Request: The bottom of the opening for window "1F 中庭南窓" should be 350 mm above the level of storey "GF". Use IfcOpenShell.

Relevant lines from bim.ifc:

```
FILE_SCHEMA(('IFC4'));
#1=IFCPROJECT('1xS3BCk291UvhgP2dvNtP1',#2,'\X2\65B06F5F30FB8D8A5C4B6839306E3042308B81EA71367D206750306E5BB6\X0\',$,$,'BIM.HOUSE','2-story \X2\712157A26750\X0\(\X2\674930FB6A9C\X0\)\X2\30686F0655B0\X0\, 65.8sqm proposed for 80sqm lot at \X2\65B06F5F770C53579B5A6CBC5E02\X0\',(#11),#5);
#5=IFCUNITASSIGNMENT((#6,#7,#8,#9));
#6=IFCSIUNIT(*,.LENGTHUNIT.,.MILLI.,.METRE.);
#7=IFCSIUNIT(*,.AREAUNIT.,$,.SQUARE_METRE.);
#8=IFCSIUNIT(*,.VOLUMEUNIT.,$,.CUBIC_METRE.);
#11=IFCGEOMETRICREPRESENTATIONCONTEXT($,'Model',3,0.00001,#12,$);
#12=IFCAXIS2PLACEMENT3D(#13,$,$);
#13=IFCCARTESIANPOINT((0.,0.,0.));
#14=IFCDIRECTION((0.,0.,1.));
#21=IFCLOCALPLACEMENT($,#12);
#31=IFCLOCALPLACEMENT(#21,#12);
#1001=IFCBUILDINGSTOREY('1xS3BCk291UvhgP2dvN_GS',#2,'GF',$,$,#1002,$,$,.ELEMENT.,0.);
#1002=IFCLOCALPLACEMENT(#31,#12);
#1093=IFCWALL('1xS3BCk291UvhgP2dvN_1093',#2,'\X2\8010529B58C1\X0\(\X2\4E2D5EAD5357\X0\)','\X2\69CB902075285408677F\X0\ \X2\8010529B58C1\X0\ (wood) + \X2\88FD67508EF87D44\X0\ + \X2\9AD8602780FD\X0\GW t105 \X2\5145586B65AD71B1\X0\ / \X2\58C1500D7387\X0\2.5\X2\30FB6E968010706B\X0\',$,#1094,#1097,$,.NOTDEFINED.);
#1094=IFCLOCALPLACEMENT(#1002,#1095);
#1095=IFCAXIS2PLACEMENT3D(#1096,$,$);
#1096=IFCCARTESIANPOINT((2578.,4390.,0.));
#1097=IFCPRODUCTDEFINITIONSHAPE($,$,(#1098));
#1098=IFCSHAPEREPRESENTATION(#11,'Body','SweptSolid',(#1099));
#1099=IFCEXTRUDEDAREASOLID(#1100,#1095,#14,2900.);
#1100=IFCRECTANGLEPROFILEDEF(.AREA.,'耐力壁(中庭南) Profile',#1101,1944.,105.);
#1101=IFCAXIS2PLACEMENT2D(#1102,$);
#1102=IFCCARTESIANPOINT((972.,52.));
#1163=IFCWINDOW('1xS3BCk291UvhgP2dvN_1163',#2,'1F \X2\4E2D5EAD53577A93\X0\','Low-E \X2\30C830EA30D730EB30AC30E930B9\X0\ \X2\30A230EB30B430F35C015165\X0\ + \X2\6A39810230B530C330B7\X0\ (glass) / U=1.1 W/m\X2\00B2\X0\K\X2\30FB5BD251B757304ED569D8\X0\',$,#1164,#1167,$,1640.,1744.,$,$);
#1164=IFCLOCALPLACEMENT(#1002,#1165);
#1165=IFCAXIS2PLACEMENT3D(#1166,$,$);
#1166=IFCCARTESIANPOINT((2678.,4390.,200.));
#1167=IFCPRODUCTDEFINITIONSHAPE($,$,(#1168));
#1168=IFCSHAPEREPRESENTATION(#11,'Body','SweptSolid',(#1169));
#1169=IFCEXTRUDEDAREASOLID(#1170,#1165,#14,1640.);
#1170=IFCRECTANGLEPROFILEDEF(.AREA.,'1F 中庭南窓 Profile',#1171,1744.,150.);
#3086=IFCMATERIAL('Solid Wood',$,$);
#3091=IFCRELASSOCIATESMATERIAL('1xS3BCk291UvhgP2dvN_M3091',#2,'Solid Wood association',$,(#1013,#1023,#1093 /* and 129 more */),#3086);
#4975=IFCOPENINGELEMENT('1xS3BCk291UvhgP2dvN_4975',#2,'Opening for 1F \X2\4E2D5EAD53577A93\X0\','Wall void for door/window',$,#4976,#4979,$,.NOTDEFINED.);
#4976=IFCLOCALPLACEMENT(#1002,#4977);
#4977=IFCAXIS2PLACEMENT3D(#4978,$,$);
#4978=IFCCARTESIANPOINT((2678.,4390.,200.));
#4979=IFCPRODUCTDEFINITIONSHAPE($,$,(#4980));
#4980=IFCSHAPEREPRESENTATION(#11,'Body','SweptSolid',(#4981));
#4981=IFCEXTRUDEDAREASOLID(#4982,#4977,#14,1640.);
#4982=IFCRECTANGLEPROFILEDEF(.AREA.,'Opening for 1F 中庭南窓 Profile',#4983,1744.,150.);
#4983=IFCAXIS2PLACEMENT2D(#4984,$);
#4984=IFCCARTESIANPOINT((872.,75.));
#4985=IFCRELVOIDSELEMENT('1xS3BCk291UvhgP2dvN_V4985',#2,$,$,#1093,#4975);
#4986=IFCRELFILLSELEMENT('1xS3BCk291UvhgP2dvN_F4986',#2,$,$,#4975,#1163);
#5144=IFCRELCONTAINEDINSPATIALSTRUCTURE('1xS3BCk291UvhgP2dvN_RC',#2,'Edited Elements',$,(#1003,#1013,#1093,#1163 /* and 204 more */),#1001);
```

```python
import numpy as np
import ifcopenshell
import ifcopenshell.api.geometry
import ifcopenshell.geom
import ifcopenshell.util.element
import ifcopenshell.util.placement
import ifcopenshell.util.shape
import ifcopenshell.util.unit

model = ifcopenshell.open("bim.ifc")
unit_scale = ifcopenshell.util.unit.calculate_unit_scale(model)

window = model.by_id(1163)
opening = window.FillsVoids[0].RelatingOpeningElement
storey = ifcopenshell.util.element.get_container(window, ifc_class="IfcBuildingStorey")
level = ifcopenshell.util.placement.get_local_placement(storey.ObjectPlacement)[2, 3]

# The opening's origin need not be at the sill, so measure its lowest point.
shape = ifcopenshell.geom.create_shape(ifcopenshell.geom.settings(), opening)
bottom = ifcopenshell.util.shape.get_shape_bottom_elevation(shape, shape.geometry) / unit_scale
dz = level + 350.0 - bottom

shift = np.array([0.0, 0.0, dz])
# The window is not placed relative to its opening, so move both.
for product in (opening, window):
    matrix = ifcopenshell.util.placement.get_local_placement(product.ObjectPlacement)
    matrix[:3, 3] += shift
    ifcopenshell.api.geometry.edit_object_placement(model, product=product, matrix=matrix, is_si=False)

print(f"moved by {dz * unit_scale:+.3f} m")

model.write("bim_v2.ifc")
```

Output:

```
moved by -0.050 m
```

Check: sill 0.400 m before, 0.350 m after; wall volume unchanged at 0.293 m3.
